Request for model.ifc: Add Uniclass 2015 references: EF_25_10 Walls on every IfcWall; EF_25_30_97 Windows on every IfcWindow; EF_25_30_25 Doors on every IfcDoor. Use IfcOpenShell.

First a look at what the model holds.

```python
import ifcopenshell

model = ifcopenshell.open("model.ifc")
print(model.schema)
print("classifications:", [c.Name for c in model.by_type("IfcClassification")])
for ifc_class in ("IfcDoor", "IfcRoof", "IfcStair", "IfcWall", "IfcWindow"):
    print(ifc_class, len(model.by_type(ifc_class)))
```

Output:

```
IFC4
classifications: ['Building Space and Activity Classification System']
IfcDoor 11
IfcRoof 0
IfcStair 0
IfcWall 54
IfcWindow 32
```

```python
import ifcopenshell
import ifcopenshell.api.classification

model = ifcopenshell.open("model.ifc")

system = ifcopenshell.api.classification.add_classification(model, classification="Uniclass 2015")

codes = {
    "IfcWall": ("EF_25_10", "Walls"),
    "IfcWindow": ("EF_25_30_97", "Windows"),
    "IfcDoor": ("EF_25_30_25", "Doors"),
}
for ifc_class, (code, name) in codes.items():
    products = model.by_type(ifc_class)
    ifcopenshell.api.classification.add_reference(
        model, products=products, classification=system, identification=code, name=name
    )
    print(code, len(products))

model.write("model-out.ifc")
```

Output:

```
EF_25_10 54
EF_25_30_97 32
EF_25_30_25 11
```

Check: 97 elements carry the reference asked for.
